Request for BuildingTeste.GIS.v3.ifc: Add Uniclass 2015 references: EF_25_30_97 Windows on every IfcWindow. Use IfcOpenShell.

First a look at what the model holds.

```python
import ifcopenshell

model = ifcopenshell.open("BuildingTeste.GIS.v3.ifc")
print(model.schema)
print("classifications:", [c.Name for c in model.by_type("IfcClassification")])
for ifc_class in ("IfcDoor", "IfcRoof", "IfcStair", "IfcWall", "IfcWindow"):
    print(ifc_class, len(model.by_type(ifc_class)))
```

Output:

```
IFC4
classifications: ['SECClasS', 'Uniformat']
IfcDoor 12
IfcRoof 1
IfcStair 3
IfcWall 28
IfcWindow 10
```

```python
import ifcopenshell
import ifcopenshell.api.classification

model = ifcopenshell.open("BuildingTeste.GIS.v3.ifc")

system = ifcopenshell.api.classification.add_classification(model, classification="Uniclass 2015")

codes = {
    "IfcWindow": ("EF_25_30_97", "Windows"),
}
for ifc_class, (code, name) in codes.items():
    products = model.by_type(ifc_class)
    ifcopenshell.api.classification.add_reference(
        model, products=products, classification=system, identification=code, name=name
    )
    print(code, len(products))

model.write("BuildingTeste.GIS.v3_rev.ifc")
```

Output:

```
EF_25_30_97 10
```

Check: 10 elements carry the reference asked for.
